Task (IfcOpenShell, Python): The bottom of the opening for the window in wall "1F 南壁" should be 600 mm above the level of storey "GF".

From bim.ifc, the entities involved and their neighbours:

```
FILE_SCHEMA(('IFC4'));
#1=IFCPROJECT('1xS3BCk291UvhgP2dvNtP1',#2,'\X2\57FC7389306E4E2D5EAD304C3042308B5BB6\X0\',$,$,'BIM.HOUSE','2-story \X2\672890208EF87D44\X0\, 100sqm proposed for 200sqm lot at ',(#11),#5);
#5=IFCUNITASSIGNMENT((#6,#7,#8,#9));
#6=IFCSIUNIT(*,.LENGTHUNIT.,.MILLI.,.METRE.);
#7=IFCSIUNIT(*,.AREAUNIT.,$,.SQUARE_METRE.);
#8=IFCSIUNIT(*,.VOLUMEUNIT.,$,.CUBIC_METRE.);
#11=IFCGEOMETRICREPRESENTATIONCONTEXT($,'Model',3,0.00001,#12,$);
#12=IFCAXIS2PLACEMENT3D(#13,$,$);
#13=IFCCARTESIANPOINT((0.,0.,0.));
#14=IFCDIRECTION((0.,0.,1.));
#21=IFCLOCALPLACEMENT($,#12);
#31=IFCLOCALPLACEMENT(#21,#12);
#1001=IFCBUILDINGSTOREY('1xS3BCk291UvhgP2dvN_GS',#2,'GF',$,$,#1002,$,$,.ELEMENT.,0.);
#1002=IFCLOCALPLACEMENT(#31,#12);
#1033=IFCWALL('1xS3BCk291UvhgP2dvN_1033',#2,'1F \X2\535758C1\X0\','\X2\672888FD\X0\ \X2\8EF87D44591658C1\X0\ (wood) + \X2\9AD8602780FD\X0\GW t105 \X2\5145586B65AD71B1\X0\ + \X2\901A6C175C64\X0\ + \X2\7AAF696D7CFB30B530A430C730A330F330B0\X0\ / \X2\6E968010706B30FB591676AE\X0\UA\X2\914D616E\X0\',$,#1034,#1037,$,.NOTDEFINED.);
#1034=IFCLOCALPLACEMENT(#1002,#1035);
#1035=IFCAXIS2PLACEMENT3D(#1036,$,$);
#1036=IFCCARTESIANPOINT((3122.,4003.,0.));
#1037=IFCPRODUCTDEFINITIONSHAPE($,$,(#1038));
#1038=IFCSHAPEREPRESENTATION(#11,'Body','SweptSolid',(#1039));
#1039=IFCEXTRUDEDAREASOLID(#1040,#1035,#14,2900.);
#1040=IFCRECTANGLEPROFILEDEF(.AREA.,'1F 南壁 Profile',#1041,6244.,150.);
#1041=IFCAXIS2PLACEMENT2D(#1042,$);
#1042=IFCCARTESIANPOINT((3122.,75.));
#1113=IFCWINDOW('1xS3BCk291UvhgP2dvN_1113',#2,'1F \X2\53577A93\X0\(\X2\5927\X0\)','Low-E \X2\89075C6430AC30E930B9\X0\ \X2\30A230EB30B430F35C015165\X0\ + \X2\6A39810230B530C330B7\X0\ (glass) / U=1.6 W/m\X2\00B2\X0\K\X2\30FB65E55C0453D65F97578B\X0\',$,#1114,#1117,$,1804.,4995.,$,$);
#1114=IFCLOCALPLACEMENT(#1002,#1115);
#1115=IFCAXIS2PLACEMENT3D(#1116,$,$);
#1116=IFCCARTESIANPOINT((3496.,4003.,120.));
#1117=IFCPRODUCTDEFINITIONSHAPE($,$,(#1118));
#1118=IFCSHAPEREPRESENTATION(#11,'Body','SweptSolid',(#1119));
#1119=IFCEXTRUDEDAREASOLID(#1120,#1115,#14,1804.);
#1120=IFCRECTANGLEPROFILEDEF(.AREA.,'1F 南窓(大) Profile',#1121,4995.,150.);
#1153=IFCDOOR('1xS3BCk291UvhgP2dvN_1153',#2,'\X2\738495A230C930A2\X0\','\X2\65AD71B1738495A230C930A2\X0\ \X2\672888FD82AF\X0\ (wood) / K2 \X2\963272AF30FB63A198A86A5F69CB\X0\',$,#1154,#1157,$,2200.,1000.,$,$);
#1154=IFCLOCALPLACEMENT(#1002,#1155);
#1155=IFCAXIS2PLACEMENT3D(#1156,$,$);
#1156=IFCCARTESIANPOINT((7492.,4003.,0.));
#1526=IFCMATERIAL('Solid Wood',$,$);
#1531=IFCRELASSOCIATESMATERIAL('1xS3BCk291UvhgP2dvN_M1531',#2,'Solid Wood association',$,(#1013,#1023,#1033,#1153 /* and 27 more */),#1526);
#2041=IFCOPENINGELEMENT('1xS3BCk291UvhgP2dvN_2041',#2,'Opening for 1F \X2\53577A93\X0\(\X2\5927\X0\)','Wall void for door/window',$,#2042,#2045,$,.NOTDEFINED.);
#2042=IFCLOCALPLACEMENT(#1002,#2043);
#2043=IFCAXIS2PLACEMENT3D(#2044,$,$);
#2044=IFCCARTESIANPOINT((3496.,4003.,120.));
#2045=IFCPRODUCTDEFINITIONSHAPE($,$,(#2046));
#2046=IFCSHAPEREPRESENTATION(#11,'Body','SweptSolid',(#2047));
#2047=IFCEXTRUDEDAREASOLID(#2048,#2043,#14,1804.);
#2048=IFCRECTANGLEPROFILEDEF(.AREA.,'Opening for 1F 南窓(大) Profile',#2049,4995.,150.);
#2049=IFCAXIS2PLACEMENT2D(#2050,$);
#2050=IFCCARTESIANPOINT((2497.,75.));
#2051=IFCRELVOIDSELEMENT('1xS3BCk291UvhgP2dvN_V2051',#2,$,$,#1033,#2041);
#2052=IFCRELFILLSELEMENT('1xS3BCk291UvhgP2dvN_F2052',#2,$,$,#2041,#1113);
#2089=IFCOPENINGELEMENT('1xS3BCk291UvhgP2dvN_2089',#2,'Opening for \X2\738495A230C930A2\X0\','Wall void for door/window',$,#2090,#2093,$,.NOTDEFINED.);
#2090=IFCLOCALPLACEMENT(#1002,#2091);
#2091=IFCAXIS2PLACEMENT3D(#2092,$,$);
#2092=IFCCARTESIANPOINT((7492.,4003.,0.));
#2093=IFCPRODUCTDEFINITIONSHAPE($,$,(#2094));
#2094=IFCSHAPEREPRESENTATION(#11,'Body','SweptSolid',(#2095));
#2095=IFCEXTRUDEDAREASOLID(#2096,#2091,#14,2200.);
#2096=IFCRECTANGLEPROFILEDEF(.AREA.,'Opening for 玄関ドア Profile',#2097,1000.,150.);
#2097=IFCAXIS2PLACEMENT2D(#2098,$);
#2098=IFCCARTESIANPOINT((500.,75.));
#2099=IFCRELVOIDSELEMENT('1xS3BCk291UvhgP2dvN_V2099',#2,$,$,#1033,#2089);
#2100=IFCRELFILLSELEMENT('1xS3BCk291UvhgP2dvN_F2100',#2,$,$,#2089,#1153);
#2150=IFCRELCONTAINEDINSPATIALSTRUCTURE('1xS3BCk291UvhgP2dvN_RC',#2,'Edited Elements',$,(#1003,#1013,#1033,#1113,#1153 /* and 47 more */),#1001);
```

```python
import numpy as np
import ifcopenshell
import ifcopenshell.api.geometry
import ifcopenshell.geom
import ifcopenshell.util.element
import ifcopenshell.util.placement
import ifcopenshell.util.shape
import ifcopenshell.util.unit

model = ifcopenshell.open("bim.ifc")
unit_scale = ifcopenshell.util.unit.calculate_unit_scale(model)

window = model.by_guid("1xS3BCk291UvhgP2dvN_1113")
opening = window.FillsVoids[0].RelatingOpeningElement
storey = ifcopenshell.util.element.get_container(window, ifc_class="IfcBuildingStorey")
level = ifcopenshell.util.placement.get_local_placement(storey.ObjectPlacement)[2, 3]

# The opening's origin need not be at the sill, so measure its lowest point.
shape = ifcopenshell.geom.create_shape(ifcopenshell.geom.settings(), opening)
bottom = ifcopenshell.util.shape.get_shape_bottom_elevation(shape, shape.geometry) / unit_scale
dz = level + 0.6 / unit_scale - bottom

shift = np.array([0.0, 0.0, dz])
# The window is not placed relative to its opening, so move both.
for product in (opening, window):
    matrix = ifcopenshell.util.placement.get_local_placement(product.ObjectPlacement)
    matrix[:3, 3] += shift
    ifcopenshell.api.geometry.edit_object_placement(model, product=product, matrix=matrix, is_si=False)

print(f"moved by {dz * unit_scale:+.3f} m")

model.write("bim_v2.ifc")
```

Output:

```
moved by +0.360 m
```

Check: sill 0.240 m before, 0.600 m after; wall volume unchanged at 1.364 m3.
